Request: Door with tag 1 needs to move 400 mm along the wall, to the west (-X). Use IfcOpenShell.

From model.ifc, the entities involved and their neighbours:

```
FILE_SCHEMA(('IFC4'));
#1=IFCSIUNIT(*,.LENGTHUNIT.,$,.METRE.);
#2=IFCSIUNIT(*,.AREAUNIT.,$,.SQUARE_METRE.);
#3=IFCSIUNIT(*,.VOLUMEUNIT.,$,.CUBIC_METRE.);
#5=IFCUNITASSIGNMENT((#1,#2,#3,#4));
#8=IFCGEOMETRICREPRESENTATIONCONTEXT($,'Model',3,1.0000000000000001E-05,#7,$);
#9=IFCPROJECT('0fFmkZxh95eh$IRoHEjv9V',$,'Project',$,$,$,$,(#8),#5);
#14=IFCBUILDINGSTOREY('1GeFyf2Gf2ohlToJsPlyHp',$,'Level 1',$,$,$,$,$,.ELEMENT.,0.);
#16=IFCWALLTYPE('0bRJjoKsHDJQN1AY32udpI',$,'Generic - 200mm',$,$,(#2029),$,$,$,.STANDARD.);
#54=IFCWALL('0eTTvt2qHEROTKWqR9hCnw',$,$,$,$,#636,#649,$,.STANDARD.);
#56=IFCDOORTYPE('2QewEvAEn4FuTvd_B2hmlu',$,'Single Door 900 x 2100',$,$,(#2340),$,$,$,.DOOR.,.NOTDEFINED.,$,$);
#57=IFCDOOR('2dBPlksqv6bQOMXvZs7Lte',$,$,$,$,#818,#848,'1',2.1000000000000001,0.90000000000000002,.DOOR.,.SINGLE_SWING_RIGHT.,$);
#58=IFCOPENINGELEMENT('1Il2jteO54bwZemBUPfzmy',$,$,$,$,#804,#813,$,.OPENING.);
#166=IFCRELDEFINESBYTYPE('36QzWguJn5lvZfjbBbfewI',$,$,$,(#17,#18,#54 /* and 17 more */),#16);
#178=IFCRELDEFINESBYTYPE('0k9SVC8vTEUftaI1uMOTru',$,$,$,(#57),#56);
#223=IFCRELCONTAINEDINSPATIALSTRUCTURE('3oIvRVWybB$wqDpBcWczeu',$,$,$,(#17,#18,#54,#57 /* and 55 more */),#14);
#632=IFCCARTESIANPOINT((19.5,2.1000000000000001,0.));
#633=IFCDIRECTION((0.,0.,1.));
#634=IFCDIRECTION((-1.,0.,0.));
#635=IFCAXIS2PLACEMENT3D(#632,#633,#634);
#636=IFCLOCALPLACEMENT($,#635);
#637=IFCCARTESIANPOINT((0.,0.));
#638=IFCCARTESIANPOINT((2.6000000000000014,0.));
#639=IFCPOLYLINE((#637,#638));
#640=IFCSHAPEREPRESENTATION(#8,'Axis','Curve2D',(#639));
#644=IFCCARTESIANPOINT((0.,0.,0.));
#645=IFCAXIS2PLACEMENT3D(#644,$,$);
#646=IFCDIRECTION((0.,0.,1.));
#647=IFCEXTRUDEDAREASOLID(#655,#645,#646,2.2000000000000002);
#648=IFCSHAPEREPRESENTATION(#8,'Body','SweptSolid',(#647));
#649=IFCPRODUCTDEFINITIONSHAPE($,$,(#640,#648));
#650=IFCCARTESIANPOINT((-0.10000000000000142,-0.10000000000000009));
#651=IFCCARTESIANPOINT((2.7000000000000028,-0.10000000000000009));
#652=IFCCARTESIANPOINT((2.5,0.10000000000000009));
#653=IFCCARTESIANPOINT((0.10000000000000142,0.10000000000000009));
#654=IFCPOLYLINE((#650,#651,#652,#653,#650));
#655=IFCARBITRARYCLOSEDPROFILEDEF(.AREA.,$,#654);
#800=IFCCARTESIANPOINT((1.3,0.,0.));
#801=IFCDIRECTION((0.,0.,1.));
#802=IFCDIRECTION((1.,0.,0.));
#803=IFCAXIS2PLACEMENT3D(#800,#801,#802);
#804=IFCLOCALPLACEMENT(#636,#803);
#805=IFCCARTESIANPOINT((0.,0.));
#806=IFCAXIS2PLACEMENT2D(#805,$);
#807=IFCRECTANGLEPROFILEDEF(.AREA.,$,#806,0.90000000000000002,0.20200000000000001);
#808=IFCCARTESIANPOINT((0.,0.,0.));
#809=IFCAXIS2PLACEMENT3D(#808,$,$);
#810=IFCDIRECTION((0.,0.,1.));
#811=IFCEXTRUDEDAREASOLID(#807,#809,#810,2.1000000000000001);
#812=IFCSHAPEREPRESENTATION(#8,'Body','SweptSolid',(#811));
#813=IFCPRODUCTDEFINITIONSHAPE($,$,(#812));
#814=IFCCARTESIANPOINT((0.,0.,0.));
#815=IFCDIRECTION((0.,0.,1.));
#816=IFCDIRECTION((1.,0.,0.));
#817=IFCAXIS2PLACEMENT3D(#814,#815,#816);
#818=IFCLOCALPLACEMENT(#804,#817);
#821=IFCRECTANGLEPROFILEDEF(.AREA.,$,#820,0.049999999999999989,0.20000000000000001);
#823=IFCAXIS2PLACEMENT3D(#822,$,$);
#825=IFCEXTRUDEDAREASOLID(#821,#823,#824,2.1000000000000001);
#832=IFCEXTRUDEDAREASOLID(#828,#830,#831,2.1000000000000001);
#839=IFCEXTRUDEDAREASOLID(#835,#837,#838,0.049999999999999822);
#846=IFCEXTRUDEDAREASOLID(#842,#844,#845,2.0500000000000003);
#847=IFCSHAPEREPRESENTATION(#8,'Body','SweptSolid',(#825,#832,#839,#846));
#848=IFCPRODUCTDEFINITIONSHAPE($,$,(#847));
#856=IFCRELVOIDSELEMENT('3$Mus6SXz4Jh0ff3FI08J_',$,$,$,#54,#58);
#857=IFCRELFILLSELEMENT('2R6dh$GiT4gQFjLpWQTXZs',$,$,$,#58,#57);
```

```python
import ifcopenshell
import ifcopenshell.api.geometry
import ifcopenshell.util.placement

model = ifcopenshell.open("model.ifc")

door = model.by_guid("2dBPlksqv6bQOMXvZs7Lte")
opening = door.FillsVoids[0].RelatingOpeningElement
wall = opening.VoidsElements[0].RelatingBuildingElement

wall_matrix = ifcopenshell.util.placement.get_local_placement(wall.ObjectPlacement)
shift = wall_matrix[:3, 0] * 0.4
before = ifcopenshell.util.placement.get_local_placement(door.ObjectPlacement)[:3, 3].copy()

# The door is placed relative to its opening, so it follows when the opening moves.
matrix = ifcopenshell.util.placement.get_local_placement(opening.ObjectPlacement)
matrix[:3, 3] += shift
ifcopenshell.api.geometry.edit_object_placement(
    model, product=opening, matrix=matrix, is_si=False, should_transform_children=True
)

after = ifcopenshell.util.placement.get_local_placement(door.ObjectPlacement)[:3, 3]
print("door moved by", (after - before).round(3) + 0.0)

model.write("model_edited.ifc")
```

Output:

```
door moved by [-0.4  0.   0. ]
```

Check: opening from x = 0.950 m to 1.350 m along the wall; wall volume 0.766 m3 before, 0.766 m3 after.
